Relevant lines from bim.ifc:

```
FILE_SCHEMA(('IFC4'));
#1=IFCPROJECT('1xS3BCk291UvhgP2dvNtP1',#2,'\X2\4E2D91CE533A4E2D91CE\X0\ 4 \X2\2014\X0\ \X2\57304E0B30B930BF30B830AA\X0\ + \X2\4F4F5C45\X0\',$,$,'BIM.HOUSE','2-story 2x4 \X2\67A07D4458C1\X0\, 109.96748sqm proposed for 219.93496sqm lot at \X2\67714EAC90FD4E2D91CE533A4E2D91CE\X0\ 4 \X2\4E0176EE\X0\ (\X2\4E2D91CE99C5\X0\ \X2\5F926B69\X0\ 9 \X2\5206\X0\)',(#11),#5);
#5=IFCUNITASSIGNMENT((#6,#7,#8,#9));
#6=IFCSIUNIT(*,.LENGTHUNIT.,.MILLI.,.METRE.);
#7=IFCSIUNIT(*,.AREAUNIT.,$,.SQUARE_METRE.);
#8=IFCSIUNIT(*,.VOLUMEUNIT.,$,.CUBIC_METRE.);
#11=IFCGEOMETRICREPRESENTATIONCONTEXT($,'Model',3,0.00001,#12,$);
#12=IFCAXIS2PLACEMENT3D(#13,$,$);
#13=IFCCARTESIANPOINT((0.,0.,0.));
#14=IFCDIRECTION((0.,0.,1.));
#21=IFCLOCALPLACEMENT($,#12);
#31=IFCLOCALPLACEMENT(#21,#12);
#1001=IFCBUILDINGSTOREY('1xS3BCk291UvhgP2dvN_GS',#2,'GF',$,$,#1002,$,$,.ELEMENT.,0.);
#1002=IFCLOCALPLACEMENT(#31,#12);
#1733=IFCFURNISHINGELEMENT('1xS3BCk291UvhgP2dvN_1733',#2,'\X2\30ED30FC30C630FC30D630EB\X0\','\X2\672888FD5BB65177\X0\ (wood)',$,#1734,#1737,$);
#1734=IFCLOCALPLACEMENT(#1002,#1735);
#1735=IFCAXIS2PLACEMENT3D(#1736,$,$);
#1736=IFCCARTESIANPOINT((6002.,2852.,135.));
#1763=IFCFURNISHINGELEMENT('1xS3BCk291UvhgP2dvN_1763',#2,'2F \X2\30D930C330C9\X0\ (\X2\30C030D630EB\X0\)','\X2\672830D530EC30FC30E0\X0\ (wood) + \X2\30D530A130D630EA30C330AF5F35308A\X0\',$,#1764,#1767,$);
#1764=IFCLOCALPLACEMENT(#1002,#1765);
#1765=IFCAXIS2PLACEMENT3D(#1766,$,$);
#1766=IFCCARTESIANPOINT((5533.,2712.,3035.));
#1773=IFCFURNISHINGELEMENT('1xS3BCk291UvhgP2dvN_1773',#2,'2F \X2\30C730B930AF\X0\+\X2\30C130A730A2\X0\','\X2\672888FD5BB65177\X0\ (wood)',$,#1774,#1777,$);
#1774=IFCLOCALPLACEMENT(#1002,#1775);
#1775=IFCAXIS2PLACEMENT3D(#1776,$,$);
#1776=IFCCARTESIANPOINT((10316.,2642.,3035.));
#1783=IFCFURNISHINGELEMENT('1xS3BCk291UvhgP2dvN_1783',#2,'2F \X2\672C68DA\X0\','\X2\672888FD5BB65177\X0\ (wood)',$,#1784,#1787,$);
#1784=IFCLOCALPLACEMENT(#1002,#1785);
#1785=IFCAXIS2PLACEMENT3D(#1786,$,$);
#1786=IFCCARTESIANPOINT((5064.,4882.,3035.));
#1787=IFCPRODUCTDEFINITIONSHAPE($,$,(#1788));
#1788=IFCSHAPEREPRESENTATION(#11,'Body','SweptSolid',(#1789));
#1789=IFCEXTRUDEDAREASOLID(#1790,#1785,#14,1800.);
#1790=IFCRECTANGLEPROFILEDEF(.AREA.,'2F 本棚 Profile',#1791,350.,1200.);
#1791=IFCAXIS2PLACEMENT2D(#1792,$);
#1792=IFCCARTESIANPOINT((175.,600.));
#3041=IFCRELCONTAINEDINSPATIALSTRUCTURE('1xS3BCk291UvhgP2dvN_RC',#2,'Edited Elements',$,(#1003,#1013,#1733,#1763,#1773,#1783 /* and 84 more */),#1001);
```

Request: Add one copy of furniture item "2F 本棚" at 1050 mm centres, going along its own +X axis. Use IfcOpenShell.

```python
import ifcopenshell
import ifcopenshell.api.geometry
import ifcopenshell.api.root
import ifcopenshell.util.element
import ifcopenshell.util.placement

model = ifcopenshell.open("bim.ifc")


def reuse_history(source, copy):
    """copy_class also copies each property set's owner history, people and application; keep the originals."""
    for rel in copy.IsDefinedBy:
        if rel.is_a("IfcRelDefinesByProperties") and (history := rel.RelatingPropertyDefinition.OwnerHistory):
            rel.RelatingPropertyDefinition.OwnerHistory = source.OwnerHistory
            ifcopenshell.util.element.remove_deep2(model, history)


source = model.by_guid("1xS3BCk291UvhgP2dvN_1783")
base = ifcopenshell.util.placement.get_local_placement(source.ObjectPlacement)
step = base[:3, 0] * 1050.0

for i in range(1, 2):
    copy = ifcopenshell.api.root.copy_class(model, product=source)
    copy.Representation = ifcopenshell.util.element.copy_deep(
        model, source.Representation, exclude=["IfcGeometricRepresentationContext", "IfcRepresentationMap"]
    )
    reuse_history(source, copy)
    matrix = base.copy()
    matrix[:3, 3] += i * step
    print("added at", matrix[:3, 3].round(3) + 0.0)
    ifcopenshell.api.geometry.edit_object_placement(model, product=copy, matrix=matrix, is_si=False)

model.write("bim_edited.ifc")
```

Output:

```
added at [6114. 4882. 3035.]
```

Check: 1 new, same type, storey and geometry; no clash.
